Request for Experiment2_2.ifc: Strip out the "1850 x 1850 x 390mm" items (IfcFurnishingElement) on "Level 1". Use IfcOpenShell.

First a look at what the model holds.

```python
import ifcopenshell
import ifcopenshell.util.element

model = ifcopenshell.open("Experiment2_2.ifc")
print(model.schema)
storey = next(s for s in model.by_type("IfcBuildingStorey") if s.Name == "Level 1")
furniture = [e for e in ifcopenshell.util.element.get_decomposition(storey) if e.is_a("IfcFurnishingElement")]
seen = {}
for e in furniture:
    element_type = ifcopenshell.util.element.get_type(e)
    name = element_type.Name if element_type not in (None, e) else None
    seen[name] = seen.get(name, 0) + 1
for name, count in sorted(seen.items(), key=str):
    print(count, "x", name)
```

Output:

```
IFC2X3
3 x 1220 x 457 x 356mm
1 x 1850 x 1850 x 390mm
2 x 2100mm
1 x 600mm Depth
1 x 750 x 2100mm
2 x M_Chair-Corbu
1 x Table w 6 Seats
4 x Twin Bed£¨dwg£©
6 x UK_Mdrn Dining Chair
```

```python
import ifcopenshell
import ifcopenshell.api.root
import ifcopenshell.util.element

model = ifcopenshell.open("Experiment2_2.ifc")

storey = next(s for s in model.by_type("IfcBuildingStorey") if s.Name == "Level 1")
furniture = [e for e in ifcopenshell.util.element.get_decomposition(storey) if e.is_a("IfcFurnishingElement")]
targets = [e for e in furniture if (t := ifcopenshell.util.element.get_type(e)) not in (None, e) and t.Name == "1850 x 1850 x 390mm"]

for e in targets:
    ifcopenshell.api.root.remove_product(model, product=e)
print(len(targets), "removed")

model.write("Experiment2_2_edited.ifc")
```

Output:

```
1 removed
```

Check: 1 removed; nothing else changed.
